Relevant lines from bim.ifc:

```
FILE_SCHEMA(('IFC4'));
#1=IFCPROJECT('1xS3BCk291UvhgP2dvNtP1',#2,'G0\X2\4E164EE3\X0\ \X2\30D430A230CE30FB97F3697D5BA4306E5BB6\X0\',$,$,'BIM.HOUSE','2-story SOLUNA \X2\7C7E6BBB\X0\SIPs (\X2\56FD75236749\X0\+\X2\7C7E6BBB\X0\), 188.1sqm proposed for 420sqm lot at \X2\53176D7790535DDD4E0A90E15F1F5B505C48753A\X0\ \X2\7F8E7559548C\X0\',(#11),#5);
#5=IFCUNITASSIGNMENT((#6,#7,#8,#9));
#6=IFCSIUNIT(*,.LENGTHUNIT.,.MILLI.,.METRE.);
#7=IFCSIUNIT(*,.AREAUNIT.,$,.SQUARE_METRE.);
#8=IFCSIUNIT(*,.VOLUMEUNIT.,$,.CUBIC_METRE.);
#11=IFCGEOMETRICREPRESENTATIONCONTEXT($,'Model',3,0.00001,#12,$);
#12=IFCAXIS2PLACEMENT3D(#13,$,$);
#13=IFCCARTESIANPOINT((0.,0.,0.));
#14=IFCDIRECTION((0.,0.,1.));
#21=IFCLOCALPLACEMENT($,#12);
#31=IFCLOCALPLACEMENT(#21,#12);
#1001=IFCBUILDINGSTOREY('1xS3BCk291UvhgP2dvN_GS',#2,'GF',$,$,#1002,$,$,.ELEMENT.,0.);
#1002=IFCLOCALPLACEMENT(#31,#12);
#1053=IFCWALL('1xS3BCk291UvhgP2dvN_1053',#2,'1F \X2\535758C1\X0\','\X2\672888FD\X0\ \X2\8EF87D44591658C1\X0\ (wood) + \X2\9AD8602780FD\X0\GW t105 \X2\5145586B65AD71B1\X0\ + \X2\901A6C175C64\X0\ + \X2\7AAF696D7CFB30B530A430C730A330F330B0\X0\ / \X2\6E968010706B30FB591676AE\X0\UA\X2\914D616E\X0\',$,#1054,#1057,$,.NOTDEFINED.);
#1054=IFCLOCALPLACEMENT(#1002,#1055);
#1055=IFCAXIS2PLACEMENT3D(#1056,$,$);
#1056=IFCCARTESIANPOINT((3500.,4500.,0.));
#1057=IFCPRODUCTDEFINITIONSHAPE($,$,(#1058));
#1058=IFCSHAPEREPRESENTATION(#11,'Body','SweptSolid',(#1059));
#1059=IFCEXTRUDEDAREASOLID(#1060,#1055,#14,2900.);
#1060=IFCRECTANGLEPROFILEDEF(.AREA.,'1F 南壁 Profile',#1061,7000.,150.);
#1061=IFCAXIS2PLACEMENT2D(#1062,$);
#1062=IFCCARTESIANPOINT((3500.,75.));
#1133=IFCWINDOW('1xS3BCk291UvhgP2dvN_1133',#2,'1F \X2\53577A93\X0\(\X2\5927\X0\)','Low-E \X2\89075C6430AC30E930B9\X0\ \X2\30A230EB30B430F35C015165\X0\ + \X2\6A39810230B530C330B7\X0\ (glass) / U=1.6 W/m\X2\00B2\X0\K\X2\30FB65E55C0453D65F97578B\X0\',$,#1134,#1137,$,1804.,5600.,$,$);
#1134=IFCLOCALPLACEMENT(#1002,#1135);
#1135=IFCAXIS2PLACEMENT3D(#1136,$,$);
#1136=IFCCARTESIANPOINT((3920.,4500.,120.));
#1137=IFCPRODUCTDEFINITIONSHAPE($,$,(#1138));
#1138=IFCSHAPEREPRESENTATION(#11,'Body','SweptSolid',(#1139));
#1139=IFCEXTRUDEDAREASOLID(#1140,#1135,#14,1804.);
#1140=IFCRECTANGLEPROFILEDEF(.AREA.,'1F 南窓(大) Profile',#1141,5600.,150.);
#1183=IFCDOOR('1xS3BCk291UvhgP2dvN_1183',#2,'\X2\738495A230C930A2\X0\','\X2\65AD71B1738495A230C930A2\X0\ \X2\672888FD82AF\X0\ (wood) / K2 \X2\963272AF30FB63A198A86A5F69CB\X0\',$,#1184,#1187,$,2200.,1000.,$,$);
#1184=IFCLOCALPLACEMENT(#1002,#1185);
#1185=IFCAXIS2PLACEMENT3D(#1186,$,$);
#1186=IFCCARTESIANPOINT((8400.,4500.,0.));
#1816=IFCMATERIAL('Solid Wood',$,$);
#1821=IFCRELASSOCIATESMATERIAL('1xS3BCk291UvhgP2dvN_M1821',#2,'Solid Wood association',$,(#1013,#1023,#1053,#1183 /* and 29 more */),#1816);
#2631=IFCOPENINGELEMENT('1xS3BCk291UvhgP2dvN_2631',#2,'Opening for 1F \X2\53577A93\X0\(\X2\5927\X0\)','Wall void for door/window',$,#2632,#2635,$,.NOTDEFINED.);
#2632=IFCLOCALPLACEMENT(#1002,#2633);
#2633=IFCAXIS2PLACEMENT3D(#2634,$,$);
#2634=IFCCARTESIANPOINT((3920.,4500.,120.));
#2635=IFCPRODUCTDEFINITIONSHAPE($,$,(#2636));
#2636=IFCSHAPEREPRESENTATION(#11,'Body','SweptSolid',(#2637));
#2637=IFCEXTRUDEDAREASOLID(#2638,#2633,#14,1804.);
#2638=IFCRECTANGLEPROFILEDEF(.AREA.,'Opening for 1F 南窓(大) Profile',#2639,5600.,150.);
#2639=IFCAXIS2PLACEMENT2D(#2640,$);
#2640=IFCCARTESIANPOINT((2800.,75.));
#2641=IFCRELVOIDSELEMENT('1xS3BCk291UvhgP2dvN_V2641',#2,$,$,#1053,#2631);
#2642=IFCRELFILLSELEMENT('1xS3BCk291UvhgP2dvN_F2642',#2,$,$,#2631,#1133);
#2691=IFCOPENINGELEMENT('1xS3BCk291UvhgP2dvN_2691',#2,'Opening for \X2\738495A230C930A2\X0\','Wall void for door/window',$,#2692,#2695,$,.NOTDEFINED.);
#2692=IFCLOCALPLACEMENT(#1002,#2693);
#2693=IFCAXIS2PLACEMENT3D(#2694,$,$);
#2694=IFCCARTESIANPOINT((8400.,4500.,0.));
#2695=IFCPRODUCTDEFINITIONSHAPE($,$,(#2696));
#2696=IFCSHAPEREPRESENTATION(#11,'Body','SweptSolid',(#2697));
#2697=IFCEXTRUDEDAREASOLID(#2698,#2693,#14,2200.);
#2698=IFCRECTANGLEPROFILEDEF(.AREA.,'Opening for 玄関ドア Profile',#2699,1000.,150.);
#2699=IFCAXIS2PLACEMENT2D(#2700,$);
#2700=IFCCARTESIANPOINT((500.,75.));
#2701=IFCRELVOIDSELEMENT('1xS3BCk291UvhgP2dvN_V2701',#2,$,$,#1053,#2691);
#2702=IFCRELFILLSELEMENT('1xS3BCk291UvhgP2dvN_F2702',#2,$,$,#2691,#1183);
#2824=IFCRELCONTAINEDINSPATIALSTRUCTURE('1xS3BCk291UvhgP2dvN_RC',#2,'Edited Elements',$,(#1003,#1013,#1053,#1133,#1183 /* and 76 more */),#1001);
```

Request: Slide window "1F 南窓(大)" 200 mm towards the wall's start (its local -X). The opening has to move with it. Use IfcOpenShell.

```python
import ifcopenshell
import ifcopenshell.api.geometry
import ifcopenshell.util.placement

model = ifcopenshell.open("bim.ifc")

window = model.by_id(1133)
opening = window.FillsVoids[0].RelatingOpeningElement
wall = opening.VoidsElements[0].RelatingBuildingElement

wall_matrix = ifcopenshell.util.placement.get_local_placement(wall.ObjectPlacement)
shift = wall_matrix[:3, 0] * -200.0
before = ifcopenshell.util.placement.get_local_placement(window.ObjectPlacement)[:3, 3].copy()

# The window is not placed relative to its opening, so move both.
for product in (opening, window):
    matrix = ifcopenshell.util.placement.get_local_placement(product.ObjectPlacement)
    matrix[:3, 3] += shift
    ifcopenshell.api.geometry.edit_object_placement(model, product=product, matrix=matrix, is_si=False)

after = ifcopenshell.util.placement.get_local_placement(window.ObjectPlacement)[:3, 3]
print("window moved by", (after - before).round(3) + 0.0)

model.write("bim_v2.ifc")
```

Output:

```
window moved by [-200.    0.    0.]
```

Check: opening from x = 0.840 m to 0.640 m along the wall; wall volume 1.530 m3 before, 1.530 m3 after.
